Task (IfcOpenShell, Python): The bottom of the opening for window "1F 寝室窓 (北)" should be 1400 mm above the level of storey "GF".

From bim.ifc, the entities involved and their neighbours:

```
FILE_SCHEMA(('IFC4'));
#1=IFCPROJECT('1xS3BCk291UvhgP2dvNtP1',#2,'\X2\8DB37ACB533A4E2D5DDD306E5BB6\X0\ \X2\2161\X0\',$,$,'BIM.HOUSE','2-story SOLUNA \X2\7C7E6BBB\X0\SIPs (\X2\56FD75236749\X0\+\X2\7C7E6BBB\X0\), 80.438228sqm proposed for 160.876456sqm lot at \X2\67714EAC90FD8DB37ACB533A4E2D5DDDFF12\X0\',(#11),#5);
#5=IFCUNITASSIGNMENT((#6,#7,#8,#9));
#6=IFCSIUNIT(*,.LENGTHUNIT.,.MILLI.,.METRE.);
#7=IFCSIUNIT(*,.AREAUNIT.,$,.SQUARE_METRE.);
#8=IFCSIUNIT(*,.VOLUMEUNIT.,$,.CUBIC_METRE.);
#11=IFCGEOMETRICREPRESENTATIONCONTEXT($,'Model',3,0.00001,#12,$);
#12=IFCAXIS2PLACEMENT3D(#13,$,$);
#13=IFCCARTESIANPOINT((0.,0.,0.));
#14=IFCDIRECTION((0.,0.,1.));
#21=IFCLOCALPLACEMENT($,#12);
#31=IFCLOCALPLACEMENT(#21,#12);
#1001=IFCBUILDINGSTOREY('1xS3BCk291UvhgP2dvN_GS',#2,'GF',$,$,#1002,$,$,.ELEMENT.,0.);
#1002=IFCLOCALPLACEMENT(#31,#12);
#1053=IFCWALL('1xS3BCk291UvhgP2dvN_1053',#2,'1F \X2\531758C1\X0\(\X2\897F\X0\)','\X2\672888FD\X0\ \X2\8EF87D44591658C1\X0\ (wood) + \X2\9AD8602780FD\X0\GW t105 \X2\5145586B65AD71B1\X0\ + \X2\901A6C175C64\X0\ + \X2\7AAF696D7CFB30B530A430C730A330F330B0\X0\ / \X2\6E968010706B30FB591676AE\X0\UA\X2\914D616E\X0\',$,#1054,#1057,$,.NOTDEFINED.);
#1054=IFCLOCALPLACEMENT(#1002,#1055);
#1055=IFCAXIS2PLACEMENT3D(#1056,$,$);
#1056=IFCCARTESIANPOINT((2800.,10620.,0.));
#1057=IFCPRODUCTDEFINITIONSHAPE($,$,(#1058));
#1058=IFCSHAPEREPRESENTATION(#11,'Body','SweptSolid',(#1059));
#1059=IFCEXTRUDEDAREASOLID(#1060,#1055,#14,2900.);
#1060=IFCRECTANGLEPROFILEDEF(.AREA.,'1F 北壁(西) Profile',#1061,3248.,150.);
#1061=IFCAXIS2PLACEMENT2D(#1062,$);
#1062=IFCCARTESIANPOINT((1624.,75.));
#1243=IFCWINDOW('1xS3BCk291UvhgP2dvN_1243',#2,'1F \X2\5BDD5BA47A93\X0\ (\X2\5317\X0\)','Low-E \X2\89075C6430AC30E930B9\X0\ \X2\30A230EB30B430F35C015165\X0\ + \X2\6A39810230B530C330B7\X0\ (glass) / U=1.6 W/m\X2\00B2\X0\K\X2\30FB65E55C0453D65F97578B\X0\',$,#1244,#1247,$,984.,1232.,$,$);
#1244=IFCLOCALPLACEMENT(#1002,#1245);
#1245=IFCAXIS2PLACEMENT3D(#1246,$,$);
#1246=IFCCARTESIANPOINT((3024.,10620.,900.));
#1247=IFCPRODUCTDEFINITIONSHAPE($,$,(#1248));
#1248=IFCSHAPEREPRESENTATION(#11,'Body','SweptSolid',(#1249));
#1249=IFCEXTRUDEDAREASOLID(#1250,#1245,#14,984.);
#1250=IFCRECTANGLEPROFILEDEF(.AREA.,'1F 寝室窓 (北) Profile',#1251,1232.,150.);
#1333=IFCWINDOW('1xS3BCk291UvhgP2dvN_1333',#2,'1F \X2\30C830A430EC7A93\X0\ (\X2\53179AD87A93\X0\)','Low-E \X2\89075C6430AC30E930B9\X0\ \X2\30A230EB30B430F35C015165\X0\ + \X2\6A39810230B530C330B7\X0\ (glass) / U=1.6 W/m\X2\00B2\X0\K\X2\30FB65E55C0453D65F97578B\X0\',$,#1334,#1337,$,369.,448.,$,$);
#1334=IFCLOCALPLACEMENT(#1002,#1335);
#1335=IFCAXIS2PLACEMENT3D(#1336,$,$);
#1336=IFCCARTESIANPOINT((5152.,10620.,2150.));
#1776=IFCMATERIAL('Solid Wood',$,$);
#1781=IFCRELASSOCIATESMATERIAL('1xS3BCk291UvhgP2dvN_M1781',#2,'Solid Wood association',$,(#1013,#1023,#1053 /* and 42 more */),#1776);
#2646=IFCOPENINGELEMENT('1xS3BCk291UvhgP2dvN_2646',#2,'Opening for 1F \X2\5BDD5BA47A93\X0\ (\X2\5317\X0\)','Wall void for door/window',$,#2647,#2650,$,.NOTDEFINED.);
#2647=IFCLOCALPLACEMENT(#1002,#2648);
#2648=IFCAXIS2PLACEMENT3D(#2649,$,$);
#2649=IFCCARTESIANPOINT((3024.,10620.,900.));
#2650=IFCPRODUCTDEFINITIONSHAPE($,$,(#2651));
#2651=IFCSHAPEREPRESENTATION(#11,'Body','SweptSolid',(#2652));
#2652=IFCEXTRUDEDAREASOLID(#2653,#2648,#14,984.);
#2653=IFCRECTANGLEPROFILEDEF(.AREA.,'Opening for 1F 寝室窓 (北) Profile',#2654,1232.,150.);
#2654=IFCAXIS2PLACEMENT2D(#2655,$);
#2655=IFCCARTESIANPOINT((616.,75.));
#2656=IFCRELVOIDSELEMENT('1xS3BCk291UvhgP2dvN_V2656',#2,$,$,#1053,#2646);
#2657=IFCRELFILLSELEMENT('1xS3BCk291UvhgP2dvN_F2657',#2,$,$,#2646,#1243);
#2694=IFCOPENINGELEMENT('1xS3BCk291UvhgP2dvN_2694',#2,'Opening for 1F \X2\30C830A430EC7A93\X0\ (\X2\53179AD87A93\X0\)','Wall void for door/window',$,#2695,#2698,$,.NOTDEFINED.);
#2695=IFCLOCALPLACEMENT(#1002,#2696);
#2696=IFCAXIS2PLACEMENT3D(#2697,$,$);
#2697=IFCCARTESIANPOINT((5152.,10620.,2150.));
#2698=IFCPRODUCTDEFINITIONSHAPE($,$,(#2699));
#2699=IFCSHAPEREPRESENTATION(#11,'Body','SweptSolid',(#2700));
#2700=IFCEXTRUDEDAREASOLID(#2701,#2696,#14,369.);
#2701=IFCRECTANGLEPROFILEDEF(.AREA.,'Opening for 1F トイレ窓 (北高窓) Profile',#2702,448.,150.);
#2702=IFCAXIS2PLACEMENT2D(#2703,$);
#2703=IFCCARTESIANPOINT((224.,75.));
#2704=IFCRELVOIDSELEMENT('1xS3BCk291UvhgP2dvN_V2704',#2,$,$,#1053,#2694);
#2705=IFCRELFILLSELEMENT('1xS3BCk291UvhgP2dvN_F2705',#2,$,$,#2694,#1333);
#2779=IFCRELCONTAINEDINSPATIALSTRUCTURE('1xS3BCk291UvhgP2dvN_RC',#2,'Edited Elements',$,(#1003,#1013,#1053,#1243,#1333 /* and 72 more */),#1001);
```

```python
import numpy as np
import ifcopenshell
import ifcopenshell.api.geometry
import ifcopenshell.geom
import ifcopenshell.util.element
import ifcopenshell.util.placement
import ifcopenshell.util.shape
import ifcopenshell.util.unit

model = ifcopenshell.open("bim.ifc")
unit_scale = ifcopenshell.util.unit.calculate_unit_scale(model)

window = model.by_guid("1xS3BCk291UvhgP2dvN_1243")
opening = window.FillsVoids[0].RelatingOpeningElement
storey = ifcopenshell.util.element.get_container(window, ifc_class="IfcBuildingStorey")
level = ifcopenshell.util.placement.get_local_placement(storey.ObjectPlacement)[2, 3]

# The opening's origin need not be at the sill, so measure its lowest point.
shape = ifcopenshell.geom.create_shape(ifcopenshell.geom.settings(), opening)
bottom = ifcopenshell.util.shape.get_shape_bottom_elevation(shape, shape.geometry) / unit_scale
dz = level + 1400.0 - bottom

shift = np.array([0.0, 0.0, dz])
# The window is not placed relative to its opening, so move both.
for product in (opening, window):
    matrix = ifcopenshell.util.placement.get_local_placement(product.ObjectPlacement)
    matrix[:3, 3] += shift
    ifcopenshell.api.geometry.edit_object_placement(model, product=product, matrix=matrix, is_si=False)

print(f"moved by {dz * unit_scale:+.3f} m")

model.write("bim-out.ifc")
```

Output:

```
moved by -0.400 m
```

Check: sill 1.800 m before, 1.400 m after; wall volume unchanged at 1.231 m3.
